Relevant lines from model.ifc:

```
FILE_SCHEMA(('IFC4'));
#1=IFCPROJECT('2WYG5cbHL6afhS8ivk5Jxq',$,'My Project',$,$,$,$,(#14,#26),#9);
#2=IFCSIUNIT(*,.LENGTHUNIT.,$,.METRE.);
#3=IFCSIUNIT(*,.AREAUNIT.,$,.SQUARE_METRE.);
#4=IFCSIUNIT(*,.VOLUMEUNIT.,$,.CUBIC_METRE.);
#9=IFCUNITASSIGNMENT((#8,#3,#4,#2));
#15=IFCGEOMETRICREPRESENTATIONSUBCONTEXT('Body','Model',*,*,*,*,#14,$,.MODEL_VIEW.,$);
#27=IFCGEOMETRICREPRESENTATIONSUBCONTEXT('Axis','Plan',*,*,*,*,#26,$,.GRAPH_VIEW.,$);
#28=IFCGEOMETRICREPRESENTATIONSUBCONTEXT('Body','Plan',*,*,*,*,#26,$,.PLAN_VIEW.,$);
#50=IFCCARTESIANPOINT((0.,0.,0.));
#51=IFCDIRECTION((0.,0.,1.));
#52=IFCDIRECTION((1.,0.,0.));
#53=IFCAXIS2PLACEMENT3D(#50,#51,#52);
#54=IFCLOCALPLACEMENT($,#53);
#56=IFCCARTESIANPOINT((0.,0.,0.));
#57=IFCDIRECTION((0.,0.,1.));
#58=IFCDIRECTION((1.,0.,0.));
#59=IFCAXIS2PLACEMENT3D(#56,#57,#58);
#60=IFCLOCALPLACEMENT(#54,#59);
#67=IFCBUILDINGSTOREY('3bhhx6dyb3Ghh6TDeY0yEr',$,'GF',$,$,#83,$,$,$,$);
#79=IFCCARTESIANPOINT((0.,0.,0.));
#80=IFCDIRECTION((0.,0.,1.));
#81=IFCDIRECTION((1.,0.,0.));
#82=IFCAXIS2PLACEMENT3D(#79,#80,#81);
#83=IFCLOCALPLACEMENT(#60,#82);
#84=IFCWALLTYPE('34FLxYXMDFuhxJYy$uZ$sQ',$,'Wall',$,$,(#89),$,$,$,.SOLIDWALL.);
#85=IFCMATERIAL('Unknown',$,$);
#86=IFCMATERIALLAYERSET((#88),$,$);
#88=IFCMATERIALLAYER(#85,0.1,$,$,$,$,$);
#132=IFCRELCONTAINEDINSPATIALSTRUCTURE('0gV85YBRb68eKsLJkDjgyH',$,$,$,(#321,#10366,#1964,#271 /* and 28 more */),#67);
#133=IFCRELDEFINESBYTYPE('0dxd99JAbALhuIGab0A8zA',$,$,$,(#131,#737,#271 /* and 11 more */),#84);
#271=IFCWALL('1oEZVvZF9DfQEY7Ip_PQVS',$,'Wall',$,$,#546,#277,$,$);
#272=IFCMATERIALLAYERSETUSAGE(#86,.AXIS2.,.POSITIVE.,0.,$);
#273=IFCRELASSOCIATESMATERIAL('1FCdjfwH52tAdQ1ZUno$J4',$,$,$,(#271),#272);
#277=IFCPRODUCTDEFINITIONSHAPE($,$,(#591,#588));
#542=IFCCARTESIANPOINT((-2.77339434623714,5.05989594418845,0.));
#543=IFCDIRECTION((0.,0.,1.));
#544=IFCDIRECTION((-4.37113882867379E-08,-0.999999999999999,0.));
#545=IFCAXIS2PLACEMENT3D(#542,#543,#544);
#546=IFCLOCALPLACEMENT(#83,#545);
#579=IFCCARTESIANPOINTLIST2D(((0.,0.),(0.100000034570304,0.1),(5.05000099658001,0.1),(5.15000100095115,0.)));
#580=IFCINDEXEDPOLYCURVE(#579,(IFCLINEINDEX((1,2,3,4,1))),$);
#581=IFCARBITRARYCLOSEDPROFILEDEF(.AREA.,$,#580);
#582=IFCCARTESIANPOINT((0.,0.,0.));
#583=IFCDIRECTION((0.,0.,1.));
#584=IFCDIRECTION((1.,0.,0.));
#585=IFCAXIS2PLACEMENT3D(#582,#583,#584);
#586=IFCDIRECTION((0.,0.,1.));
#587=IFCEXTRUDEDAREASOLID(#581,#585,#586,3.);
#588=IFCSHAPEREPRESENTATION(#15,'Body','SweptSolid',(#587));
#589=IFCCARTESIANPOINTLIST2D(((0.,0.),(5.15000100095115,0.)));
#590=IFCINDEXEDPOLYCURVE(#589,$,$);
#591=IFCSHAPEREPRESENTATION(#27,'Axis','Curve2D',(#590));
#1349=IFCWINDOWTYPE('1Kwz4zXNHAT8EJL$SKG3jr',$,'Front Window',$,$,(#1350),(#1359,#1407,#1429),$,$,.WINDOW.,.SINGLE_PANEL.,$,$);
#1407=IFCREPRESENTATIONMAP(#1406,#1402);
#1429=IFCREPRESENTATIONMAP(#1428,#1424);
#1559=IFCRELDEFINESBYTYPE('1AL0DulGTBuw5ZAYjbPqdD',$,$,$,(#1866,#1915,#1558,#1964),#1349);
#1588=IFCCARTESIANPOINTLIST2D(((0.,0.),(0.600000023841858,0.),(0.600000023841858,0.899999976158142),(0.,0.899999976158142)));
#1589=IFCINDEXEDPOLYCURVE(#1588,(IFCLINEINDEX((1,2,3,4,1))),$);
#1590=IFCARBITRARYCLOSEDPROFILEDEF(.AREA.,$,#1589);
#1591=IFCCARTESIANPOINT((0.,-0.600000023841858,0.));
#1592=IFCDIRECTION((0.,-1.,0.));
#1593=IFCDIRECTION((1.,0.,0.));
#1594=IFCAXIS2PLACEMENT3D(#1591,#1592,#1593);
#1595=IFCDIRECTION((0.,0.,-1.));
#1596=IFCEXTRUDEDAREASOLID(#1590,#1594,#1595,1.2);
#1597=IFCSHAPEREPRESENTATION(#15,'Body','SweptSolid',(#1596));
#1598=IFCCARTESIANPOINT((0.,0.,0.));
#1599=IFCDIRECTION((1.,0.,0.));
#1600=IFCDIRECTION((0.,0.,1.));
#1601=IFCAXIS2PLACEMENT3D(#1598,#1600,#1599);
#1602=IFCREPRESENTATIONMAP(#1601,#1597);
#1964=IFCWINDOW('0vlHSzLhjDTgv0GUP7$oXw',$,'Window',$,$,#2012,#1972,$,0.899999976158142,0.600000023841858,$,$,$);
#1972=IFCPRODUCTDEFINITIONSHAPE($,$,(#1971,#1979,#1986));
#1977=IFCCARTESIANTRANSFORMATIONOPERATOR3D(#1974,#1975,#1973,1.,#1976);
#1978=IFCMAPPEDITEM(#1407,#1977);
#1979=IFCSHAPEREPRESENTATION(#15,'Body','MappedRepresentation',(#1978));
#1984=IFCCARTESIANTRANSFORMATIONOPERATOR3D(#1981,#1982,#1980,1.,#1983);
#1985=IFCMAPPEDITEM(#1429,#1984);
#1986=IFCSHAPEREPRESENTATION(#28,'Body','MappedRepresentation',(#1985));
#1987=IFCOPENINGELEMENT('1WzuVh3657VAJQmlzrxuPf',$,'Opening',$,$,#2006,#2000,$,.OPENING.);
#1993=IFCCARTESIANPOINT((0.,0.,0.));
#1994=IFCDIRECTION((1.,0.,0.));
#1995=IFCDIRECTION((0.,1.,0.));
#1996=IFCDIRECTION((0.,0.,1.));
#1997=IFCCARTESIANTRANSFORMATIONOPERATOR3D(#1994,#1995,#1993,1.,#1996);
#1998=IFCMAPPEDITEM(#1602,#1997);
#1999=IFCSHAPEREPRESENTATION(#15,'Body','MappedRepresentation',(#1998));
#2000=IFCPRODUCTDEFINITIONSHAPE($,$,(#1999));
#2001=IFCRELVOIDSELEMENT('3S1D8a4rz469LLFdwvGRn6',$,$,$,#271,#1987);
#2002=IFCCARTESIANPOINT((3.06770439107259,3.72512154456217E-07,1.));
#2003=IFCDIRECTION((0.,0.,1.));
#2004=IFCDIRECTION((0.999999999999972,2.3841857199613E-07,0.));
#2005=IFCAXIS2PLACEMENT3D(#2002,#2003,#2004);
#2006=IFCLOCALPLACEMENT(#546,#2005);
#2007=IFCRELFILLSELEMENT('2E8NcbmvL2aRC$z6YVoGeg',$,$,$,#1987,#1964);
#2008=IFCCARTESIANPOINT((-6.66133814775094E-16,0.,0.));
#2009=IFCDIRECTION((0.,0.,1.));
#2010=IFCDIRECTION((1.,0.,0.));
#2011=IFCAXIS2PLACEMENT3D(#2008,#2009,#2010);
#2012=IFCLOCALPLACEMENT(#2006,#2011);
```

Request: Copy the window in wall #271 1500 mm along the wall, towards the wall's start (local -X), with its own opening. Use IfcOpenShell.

```python
import ifcopenshell
import ifcopenshell.api.feature
import ifcopenshell.api.geometry
import ifcopenshell.api.root
import ifcopenshell.geom
import ifcopenshell.util.element
import ifcopenshell.util.placement
import ifcopenshell.util.shape
import ifcopenshell.util.unit

model = ifcopenshell.open("model.ifc")
unit_scale = ifcopenshell.util.unit.calculate_unit_scale(model)
settings = ifcopenshell.geom.settings()


def volume(element):
    """Net volume in cubic metres, openings subtracted."""
    shape = ifcopenshell.geom.create_shape(settings, element)
    return ifcopenshell.util.shape.get_volume(shape.geometry)


window = model.by_guid("0vlHSzLhjDTgv0GUP7$oXw")
opening = window.FillsVoids[0].RelatingOpeningElement
wall = opening.VoidsElements[0].RelatingBuildingElement
before = volume(wall)
shift = ifcopenshell.util.placement.get_local_placement(wall.ObjectPlacement)[:3, 0] * -1.5 / unit_scale

# copy_class copies the void relationship, type, container and properties, but no geometry.
new_opening = ifcopenshell.api.root.copy_class(model, product=opening)
new_opening.Representation = ifcopenshell.util.element.copy_deep(
    model, opening.Representation, exclude=["IfcGeometricRepresentationContext", "IfcRepresentationMap"]
)
new_window = ifcopenshell.api.root.copy_class(model, product=window)
new_window.Representation = ifcopenshell.util.element.copy_deep(
    model, window.Representation, exclude=["IfcGeometricRepresentationContext", "IfcRepresentationMap"]
)
ifcopenshell.api.feature.add_filling(model, opening=new_opening, element=new_window)

for old, new in ((opening, new_opening), (window, new_window)):
    matrix = ifcopenshell.util.placement.get_local_placement(old.ObjectPlacement)
    matrix[:3, 3] += shift
    ifcopenshell.api.geometry.edit_object_placement(model, product=new, matrix=matrix, is_si=False)

after = volume(wall)

print(f"wall volume {before:.3f} -> {after:.3f} m3")

model.write("model_updated.ifc")
```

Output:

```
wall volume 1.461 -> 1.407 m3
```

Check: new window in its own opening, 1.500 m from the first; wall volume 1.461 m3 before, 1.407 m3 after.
